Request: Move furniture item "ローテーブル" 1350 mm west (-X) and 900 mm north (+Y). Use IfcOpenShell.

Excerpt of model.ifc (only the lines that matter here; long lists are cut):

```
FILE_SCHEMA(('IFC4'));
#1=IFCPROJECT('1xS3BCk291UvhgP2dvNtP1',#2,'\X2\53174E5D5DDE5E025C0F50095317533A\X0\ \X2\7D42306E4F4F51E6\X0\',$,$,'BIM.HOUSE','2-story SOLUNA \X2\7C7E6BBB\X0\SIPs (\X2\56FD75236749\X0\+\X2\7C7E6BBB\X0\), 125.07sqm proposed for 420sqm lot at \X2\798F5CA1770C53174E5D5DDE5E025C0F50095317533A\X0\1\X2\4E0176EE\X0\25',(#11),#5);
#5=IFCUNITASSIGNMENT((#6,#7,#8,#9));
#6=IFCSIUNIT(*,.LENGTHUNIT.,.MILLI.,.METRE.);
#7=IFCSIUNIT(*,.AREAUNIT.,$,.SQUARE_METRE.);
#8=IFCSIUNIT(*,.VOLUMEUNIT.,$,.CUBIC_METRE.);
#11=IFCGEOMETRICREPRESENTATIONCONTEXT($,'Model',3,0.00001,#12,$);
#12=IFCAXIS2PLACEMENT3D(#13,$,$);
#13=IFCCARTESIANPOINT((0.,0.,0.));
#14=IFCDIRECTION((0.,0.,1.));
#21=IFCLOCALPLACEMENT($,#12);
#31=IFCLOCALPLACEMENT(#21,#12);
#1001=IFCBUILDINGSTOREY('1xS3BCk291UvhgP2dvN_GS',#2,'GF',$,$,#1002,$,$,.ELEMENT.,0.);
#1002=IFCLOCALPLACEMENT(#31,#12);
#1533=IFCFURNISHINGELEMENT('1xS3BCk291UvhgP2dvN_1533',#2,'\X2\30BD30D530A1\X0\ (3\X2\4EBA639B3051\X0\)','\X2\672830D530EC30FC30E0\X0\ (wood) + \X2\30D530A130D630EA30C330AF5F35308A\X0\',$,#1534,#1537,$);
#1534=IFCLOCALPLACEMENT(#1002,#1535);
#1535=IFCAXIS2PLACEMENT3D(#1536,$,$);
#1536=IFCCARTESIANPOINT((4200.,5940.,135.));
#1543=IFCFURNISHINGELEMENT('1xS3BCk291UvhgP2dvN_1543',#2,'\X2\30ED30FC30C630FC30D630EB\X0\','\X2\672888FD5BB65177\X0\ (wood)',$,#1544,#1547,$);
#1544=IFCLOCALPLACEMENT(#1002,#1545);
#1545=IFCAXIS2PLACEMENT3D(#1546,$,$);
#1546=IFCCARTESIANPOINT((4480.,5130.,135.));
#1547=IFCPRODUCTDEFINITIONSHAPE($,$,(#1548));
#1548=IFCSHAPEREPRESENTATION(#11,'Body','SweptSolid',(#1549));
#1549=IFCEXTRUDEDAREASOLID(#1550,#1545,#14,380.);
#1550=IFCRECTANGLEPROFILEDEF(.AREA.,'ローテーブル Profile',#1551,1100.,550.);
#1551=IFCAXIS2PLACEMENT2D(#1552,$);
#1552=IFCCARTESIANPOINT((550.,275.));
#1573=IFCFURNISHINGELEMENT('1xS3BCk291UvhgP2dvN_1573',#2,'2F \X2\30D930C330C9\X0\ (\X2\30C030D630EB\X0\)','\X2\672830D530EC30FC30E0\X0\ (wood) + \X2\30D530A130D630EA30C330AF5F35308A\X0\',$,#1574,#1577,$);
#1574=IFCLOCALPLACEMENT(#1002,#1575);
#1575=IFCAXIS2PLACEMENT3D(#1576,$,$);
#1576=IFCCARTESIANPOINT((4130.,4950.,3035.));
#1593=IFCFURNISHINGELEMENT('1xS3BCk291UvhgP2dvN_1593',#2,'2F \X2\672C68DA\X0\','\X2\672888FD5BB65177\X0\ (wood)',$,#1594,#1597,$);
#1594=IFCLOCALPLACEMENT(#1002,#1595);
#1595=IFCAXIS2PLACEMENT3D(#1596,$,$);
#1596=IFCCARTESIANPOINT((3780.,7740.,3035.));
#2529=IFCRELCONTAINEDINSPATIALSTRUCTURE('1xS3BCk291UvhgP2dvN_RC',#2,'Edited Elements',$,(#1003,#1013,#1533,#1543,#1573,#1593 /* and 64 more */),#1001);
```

```python
import ifcopenshell
import ifcopenshell.api.geometry
import ifcopenshell.util.placement
import ifcopenshell.util.unit

model = ifcopenshell.open("model.ifc")
unit_scale = ifcopenshell.util.unit.calculate_unit_scale(model)

item = model.by_guid("1xS3BCk291UvhgP2dvN_1543")
matrix = ifcopenshell.util.placement.get_local_placement(item.ObjectPlacement)
matrix[0, 3] -= 1.35 / unit_scale
matrix[1, 3] += 0.9 / unit_scale
ifcopenshell.api.geometry.edit_object_placement(model, product=item, matrix=matrix, is_si=False)

print(ifcopenshell.util.placement.get_local_placement(item.ObjectPlacement).round(3) + 0.0)

model.write("model-out.ifc")
```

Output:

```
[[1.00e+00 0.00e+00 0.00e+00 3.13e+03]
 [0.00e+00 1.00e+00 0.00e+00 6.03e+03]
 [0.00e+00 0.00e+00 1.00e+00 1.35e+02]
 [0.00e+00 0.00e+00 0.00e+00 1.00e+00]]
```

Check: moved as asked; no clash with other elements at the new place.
